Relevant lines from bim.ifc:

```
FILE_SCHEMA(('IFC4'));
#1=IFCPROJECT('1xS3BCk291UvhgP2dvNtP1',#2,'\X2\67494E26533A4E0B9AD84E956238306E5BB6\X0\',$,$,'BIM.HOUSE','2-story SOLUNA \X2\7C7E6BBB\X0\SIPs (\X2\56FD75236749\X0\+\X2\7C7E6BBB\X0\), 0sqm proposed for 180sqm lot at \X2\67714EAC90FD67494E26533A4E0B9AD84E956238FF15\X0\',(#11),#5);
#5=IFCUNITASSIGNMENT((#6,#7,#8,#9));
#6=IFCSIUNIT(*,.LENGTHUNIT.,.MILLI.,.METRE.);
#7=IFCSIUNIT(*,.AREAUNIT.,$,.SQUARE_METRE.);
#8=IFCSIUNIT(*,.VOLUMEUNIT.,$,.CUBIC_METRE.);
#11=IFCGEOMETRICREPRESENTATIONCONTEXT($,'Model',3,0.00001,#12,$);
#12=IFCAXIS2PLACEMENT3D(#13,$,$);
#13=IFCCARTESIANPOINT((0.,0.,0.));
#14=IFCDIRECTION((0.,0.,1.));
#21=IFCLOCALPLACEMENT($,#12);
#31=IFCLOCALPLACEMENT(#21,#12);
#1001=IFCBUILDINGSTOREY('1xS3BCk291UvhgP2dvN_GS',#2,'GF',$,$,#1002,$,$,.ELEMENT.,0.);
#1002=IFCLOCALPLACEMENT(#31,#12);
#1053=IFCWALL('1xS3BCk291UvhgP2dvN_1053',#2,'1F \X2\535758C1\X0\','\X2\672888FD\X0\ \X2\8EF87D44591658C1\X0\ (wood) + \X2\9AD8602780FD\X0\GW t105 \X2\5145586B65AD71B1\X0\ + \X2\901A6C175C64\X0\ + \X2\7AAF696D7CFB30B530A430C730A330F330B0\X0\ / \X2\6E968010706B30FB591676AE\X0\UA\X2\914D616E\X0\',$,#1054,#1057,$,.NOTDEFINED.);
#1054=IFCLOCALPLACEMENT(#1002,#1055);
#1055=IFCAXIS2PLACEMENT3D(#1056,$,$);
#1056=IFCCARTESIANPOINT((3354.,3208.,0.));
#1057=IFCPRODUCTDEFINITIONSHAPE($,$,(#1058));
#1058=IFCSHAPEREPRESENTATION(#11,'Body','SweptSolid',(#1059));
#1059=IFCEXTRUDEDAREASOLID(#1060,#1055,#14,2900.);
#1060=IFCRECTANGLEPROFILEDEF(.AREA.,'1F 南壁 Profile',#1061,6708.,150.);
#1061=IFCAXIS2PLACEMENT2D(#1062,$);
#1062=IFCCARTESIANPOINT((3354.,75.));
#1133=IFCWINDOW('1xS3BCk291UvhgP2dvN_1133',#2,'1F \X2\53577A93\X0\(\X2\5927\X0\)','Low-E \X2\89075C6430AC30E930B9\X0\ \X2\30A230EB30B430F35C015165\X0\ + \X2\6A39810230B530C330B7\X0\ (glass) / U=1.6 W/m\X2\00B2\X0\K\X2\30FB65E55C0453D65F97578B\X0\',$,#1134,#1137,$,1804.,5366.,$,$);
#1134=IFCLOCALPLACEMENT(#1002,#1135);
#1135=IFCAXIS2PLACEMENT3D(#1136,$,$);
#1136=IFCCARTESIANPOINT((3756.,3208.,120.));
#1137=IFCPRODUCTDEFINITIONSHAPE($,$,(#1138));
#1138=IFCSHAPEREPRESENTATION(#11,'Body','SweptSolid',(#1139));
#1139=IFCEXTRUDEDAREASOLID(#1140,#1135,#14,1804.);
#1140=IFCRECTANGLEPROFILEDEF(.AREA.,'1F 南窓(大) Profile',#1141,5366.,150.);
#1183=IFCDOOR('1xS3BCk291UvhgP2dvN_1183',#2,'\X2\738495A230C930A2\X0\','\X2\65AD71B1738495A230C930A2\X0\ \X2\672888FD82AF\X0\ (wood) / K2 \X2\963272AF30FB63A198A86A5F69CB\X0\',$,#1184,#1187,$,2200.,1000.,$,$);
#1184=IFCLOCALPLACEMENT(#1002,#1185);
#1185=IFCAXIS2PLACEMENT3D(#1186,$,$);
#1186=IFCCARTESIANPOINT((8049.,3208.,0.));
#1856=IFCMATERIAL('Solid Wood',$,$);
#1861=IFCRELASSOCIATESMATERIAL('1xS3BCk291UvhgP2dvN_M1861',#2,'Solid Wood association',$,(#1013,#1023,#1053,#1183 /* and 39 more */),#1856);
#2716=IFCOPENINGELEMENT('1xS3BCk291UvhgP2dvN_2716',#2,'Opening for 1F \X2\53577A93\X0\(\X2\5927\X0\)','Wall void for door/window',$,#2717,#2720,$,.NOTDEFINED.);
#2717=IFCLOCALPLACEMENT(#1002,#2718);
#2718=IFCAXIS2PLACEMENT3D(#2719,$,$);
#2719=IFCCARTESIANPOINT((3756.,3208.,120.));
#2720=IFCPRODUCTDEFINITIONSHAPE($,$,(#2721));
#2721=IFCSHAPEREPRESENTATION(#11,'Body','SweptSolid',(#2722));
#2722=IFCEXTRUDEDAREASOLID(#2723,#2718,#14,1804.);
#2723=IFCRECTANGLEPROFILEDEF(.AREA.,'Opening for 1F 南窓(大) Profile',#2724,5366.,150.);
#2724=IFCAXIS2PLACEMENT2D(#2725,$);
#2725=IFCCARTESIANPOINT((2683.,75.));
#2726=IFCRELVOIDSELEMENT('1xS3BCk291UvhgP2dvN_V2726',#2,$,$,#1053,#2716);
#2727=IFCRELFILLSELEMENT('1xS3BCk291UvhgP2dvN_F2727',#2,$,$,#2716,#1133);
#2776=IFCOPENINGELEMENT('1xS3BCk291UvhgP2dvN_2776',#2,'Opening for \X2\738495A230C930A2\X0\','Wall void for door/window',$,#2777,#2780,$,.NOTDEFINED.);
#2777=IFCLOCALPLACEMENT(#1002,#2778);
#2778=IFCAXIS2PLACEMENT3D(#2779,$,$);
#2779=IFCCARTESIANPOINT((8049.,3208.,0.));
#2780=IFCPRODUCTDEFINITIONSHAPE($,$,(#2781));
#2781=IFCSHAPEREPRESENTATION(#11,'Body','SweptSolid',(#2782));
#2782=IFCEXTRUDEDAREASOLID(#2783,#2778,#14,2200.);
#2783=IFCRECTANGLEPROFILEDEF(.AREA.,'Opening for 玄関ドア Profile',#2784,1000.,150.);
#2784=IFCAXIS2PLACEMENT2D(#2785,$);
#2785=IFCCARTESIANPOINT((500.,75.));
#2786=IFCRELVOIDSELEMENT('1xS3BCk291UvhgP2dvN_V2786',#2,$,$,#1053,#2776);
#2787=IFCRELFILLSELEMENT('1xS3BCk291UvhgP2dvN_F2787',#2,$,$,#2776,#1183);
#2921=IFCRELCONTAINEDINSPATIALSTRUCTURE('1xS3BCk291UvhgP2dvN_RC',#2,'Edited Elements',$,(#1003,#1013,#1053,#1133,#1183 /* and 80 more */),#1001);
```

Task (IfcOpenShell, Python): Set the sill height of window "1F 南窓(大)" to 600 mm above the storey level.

```python
import numpy as np
import ifcopenshell
import ifcopenshell.api.geometry
import ifcopenshell.geom
import ifcopenshell.util.element
import ifcopenshell.util.placement
import ifcopenshell.util.shape
import ifcopenshell.util.unit

model = ifcopenshell.open("bim.ifc")
unit_scale = ifcopenshell.util.unit.calculate_unit_scale(model)

window = model.by_guid("1xS3BCk291UvhgP2dvN_1133")
opening = window.FillsVoids[0].RelatingOpeningElement
storey = ifcopenshell.util.element.get_container(window, ifc_class="IfcBuildingStorey")
level = ifcopenshell.util.placement.get_local_placement(storey.ObjectPlacement)[2, 3]

# The opening's origin need not be at the sill, so measure its lowest point.
shape = ifcopenshell.geom.create_shape(ifcopenshell.geom.settings(), opening)
bottom = ifcopenshell.util.shape.get_shape_bottom_elevation(shape, shape.geometry) / unit_scale
dz = level + 0.6 / unit_scale - bottom

shift = np.array([0.0, 0.0, dz])
# The window is not placed relative to its opening, so move both.
for product in (opening, window):
    matrix = ifcopenshell.util.placement.get_local_placement(product.ObjectPlacement)
    matrix[:3, 3] += shift
    ifcopenshell.api.geometry.edit_object_placement(model, product=product, matrix=matrix, is_si=False)

print(f"moved by {dz * unit_scale:+.3f} m")

model.write("bim_edited.ifc")
```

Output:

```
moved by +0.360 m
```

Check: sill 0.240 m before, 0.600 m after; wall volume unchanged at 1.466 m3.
